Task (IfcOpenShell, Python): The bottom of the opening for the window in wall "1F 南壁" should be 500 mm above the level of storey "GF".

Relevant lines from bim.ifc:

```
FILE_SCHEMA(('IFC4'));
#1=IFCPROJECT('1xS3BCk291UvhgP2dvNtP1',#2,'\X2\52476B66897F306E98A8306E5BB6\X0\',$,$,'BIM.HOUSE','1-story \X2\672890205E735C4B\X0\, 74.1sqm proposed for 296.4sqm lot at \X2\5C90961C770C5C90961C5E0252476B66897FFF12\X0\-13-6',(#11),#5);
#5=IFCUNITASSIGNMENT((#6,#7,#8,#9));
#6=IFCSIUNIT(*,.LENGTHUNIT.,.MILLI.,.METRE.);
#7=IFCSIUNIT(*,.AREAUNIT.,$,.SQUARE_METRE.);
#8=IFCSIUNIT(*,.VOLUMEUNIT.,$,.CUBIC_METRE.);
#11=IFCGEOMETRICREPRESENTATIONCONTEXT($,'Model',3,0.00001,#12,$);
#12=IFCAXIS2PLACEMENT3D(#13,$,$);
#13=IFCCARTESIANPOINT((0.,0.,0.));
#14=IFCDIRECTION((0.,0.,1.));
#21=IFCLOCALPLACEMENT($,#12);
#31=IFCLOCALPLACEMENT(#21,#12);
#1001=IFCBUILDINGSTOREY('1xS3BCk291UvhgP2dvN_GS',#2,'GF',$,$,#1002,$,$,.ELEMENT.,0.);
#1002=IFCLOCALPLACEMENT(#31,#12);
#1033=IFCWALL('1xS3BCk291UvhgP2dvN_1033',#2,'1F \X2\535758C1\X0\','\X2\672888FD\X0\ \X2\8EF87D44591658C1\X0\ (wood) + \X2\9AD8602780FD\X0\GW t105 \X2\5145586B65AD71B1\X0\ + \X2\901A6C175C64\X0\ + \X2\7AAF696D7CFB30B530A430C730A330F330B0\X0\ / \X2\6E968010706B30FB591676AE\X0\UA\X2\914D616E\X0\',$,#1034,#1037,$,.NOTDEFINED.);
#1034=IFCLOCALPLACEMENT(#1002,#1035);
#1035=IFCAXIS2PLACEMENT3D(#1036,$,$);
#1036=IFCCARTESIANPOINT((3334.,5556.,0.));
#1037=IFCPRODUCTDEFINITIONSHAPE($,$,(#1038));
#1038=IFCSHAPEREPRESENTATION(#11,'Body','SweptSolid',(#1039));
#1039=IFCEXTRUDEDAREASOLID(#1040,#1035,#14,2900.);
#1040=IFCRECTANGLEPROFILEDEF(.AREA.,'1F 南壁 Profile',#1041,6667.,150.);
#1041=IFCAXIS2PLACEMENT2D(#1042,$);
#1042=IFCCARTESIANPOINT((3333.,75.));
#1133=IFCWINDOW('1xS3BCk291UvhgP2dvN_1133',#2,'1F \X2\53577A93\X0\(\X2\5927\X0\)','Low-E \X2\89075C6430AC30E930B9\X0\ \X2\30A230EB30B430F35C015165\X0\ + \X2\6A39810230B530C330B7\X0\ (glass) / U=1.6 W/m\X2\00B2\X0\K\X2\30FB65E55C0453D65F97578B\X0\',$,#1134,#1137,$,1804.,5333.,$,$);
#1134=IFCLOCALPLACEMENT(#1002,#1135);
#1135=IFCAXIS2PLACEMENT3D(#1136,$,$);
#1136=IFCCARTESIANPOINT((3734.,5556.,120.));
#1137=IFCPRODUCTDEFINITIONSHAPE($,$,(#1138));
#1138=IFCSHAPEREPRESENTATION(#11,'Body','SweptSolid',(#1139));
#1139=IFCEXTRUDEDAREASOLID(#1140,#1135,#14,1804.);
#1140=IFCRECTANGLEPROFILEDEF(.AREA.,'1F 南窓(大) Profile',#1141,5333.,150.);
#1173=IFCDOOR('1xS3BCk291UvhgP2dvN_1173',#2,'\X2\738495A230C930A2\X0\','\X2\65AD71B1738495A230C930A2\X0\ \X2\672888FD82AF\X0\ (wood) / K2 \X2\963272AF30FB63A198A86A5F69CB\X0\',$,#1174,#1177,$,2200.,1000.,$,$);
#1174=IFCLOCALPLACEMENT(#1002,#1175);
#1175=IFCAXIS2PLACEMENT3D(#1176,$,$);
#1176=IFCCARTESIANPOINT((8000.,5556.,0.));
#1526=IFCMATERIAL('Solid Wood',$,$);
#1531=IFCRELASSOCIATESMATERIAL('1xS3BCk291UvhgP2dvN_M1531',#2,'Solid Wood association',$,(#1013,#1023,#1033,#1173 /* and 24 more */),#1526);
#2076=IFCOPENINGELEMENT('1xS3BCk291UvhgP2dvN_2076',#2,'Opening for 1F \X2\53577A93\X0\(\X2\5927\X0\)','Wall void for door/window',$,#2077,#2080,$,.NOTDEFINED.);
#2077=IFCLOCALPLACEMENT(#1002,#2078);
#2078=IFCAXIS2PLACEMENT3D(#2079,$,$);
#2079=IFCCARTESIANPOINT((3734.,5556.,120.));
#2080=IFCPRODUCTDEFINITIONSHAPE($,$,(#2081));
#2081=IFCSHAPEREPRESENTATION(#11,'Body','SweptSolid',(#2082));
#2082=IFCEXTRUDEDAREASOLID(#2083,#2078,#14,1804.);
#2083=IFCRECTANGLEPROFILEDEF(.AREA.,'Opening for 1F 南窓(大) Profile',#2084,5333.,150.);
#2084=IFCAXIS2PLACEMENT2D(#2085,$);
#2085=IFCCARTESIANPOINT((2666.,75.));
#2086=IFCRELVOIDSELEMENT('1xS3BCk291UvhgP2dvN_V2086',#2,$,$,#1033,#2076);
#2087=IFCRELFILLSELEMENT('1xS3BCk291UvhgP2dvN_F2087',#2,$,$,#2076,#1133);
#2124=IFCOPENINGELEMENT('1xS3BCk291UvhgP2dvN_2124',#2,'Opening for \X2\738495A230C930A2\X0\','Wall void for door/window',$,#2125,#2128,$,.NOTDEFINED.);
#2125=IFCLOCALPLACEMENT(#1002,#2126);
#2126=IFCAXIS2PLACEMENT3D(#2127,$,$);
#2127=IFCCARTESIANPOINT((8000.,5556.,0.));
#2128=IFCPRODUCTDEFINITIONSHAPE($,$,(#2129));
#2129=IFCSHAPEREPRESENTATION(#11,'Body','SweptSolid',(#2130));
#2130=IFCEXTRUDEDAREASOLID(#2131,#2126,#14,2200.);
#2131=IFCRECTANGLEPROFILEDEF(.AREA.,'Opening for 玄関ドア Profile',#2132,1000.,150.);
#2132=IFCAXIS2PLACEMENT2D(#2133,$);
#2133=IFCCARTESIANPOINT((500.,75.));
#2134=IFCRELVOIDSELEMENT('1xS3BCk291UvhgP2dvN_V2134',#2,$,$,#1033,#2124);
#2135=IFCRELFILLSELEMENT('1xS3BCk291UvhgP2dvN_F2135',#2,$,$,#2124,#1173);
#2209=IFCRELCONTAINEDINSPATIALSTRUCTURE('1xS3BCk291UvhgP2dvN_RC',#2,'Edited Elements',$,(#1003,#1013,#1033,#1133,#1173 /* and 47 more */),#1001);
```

```python
import numpy as np
import ifcopenshell
import ifcopenshell.api.geometry
import ifcopenshell.geom
import ifcopenshell.util.element
import ifcopenshell.util.placement
import ifcopenshell.util.shape
import ifcopenshell.util.unit

model = ifcopenshell.open("bim.ifc")
unit_scale = ifcopenshell.util.unit.calculate_unit_scale(model)

window = model.by_id(1133)
opening = window.FillsVoids[0].RelatingOpeningElement
storey = ifcopenshell.util.element.get_container(window, ifc_class="IfcBuildingStorey")
level = ifcopenshell.util.placement.get_local_placement(storey.ObjectPlacement)[2, 3]

# The opening's origin need not be at the sill, so measure its lowest point.
shape = ifcopenshell.geom.create_shape(ifcopenshell.geom.settings(), opening)
bottom = ifcopenshell.util.shape.get_shape_bottom_elevation(shape, shape.geometry) / unit_scale
dz = level + 0.5 / unit_scale - bottom

shift = np.array([0.0, 0.0, dz])
# The window is not placed relative to its opening, so move both.
for product in (opening, window):
    matrix = ifcopenshell.util.placement.get_local_placement(product.ObjectPlacement)
    matrix[:3, 3] += shift
    ifcopenshell.api.geometry.edit_object_placement(model, product=product, matrix=matrix, is_si=False)

print(f"moved by {dz * unit_scale:+.3f} m")

model.write("bim_v2.ifc")
```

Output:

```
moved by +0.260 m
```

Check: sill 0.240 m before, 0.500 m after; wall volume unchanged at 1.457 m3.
